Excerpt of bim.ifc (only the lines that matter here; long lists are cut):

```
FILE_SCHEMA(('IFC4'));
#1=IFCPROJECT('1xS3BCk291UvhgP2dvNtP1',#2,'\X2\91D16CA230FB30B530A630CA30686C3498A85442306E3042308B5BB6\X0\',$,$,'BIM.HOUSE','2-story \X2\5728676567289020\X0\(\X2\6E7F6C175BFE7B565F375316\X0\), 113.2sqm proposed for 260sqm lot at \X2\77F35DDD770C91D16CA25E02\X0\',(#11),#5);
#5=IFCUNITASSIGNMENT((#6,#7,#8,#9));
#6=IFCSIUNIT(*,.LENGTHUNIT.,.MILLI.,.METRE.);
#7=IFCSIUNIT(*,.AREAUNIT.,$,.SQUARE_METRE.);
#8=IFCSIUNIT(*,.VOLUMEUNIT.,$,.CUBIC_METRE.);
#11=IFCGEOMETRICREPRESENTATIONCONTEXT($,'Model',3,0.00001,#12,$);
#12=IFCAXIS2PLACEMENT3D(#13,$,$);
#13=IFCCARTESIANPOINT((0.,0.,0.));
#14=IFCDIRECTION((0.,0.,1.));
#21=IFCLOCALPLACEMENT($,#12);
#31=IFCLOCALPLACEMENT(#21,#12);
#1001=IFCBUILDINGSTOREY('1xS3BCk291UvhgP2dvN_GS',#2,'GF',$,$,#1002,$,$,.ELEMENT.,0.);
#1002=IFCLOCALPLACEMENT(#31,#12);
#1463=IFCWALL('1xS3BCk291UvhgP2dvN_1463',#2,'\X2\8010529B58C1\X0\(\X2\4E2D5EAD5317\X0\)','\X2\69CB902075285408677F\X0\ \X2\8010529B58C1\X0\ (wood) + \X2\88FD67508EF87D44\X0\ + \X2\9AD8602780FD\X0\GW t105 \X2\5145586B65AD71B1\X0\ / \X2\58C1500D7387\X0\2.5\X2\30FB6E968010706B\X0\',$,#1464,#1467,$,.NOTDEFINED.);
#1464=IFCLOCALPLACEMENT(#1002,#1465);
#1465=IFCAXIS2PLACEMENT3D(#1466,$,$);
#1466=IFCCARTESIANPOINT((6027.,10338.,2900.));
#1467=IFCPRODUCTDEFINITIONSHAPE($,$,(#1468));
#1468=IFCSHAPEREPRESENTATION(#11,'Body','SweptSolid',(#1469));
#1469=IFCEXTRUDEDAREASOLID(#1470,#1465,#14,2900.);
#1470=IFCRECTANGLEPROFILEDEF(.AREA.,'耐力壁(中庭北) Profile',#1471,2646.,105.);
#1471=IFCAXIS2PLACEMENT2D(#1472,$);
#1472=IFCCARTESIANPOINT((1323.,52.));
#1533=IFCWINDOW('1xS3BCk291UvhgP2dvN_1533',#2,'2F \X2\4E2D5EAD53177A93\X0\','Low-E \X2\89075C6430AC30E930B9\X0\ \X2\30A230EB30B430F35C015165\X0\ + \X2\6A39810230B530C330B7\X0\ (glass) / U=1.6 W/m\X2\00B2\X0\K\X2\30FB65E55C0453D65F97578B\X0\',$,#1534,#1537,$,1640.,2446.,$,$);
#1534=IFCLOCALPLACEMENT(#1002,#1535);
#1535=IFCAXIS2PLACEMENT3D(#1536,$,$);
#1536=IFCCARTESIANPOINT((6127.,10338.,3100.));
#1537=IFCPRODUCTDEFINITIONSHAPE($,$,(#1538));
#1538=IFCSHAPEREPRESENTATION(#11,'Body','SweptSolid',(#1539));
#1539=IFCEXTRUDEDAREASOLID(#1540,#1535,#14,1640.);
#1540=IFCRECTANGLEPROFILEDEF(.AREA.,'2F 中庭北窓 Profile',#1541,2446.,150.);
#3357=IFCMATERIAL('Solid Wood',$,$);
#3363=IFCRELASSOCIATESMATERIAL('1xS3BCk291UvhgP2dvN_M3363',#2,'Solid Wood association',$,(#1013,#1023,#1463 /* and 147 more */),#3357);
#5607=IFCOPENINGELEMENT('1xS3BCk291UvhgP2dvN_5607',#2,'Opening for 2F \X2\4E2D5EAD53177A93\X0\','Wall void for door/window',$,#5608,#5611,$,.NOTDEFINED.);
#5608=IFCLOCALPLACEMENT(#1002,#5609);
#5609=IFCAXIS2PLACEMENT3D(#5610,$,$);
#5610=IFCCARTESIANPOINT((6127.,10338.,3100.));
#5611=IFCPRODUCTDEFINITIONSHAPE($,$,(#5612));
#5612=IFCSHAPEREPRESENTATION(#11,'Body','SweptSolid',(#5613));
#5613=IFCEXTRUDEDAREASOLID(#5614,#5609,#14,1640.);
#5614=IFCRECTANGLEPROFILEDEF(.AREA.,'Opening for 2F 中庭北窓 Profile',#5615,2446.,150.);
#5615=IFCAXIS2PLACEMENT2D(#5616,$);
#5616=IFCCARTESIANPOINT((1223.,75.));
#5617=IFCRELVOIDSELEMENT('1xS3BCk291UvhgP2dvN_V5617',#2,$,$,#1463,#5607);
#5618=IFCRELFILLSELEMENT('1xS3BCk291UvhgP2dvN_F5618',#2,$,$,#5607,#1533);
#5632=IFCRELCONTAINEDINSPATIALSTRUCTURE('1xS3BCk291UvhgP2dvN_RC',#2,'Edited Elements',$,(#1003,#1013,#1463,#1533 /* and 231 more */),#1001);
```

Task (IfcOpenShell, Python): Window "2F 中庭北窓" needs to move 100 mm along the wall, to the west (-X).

```python
import ifcopenshell
import ifcopenshell.api.geometry
import ifcopenshell.util.placement

model = ifcopenshell.open("bim.ifc")

window = model.by_guid("1xS3BCk291UvhgP2dvN_1533")
opening = window.FillsVoids[0].RelatingOpeningElement
wall = opening.VoidsElements[0].RelatingBuildingElement

wall_matrix = ifcopenshell.util.placement.get_local_placement(wall.ObjectPlacement)
shift = wall_matrix[:3, 0] * -100.0
before = ifcopenshell.util.placement.get_local_placement(window.ObjectPlacement)[:3, 3].copy()

# The window is not placed relative to its opening, so move both.
for product in (opening, window):
    matrix = ifcopenshell.util.placement.get_local_placement(product.ObjectPlacement)
    matrix[:3, 3] += shift
    ifcopenshell.api.geometry.edit_object_placement(model, product=product, matrix=matrix, is_si=False)

after = ifcopenshell.util.placement.get_local_placement(window.ObjectPlacement)[:3, 3]
print("window moved by", (after - before).round(3) + 0.0)

model.write("bim_v2.ifc")
```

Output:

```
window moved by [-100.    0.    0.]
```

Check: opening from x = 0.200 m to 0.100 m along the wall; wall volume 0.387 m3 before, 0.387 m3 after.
